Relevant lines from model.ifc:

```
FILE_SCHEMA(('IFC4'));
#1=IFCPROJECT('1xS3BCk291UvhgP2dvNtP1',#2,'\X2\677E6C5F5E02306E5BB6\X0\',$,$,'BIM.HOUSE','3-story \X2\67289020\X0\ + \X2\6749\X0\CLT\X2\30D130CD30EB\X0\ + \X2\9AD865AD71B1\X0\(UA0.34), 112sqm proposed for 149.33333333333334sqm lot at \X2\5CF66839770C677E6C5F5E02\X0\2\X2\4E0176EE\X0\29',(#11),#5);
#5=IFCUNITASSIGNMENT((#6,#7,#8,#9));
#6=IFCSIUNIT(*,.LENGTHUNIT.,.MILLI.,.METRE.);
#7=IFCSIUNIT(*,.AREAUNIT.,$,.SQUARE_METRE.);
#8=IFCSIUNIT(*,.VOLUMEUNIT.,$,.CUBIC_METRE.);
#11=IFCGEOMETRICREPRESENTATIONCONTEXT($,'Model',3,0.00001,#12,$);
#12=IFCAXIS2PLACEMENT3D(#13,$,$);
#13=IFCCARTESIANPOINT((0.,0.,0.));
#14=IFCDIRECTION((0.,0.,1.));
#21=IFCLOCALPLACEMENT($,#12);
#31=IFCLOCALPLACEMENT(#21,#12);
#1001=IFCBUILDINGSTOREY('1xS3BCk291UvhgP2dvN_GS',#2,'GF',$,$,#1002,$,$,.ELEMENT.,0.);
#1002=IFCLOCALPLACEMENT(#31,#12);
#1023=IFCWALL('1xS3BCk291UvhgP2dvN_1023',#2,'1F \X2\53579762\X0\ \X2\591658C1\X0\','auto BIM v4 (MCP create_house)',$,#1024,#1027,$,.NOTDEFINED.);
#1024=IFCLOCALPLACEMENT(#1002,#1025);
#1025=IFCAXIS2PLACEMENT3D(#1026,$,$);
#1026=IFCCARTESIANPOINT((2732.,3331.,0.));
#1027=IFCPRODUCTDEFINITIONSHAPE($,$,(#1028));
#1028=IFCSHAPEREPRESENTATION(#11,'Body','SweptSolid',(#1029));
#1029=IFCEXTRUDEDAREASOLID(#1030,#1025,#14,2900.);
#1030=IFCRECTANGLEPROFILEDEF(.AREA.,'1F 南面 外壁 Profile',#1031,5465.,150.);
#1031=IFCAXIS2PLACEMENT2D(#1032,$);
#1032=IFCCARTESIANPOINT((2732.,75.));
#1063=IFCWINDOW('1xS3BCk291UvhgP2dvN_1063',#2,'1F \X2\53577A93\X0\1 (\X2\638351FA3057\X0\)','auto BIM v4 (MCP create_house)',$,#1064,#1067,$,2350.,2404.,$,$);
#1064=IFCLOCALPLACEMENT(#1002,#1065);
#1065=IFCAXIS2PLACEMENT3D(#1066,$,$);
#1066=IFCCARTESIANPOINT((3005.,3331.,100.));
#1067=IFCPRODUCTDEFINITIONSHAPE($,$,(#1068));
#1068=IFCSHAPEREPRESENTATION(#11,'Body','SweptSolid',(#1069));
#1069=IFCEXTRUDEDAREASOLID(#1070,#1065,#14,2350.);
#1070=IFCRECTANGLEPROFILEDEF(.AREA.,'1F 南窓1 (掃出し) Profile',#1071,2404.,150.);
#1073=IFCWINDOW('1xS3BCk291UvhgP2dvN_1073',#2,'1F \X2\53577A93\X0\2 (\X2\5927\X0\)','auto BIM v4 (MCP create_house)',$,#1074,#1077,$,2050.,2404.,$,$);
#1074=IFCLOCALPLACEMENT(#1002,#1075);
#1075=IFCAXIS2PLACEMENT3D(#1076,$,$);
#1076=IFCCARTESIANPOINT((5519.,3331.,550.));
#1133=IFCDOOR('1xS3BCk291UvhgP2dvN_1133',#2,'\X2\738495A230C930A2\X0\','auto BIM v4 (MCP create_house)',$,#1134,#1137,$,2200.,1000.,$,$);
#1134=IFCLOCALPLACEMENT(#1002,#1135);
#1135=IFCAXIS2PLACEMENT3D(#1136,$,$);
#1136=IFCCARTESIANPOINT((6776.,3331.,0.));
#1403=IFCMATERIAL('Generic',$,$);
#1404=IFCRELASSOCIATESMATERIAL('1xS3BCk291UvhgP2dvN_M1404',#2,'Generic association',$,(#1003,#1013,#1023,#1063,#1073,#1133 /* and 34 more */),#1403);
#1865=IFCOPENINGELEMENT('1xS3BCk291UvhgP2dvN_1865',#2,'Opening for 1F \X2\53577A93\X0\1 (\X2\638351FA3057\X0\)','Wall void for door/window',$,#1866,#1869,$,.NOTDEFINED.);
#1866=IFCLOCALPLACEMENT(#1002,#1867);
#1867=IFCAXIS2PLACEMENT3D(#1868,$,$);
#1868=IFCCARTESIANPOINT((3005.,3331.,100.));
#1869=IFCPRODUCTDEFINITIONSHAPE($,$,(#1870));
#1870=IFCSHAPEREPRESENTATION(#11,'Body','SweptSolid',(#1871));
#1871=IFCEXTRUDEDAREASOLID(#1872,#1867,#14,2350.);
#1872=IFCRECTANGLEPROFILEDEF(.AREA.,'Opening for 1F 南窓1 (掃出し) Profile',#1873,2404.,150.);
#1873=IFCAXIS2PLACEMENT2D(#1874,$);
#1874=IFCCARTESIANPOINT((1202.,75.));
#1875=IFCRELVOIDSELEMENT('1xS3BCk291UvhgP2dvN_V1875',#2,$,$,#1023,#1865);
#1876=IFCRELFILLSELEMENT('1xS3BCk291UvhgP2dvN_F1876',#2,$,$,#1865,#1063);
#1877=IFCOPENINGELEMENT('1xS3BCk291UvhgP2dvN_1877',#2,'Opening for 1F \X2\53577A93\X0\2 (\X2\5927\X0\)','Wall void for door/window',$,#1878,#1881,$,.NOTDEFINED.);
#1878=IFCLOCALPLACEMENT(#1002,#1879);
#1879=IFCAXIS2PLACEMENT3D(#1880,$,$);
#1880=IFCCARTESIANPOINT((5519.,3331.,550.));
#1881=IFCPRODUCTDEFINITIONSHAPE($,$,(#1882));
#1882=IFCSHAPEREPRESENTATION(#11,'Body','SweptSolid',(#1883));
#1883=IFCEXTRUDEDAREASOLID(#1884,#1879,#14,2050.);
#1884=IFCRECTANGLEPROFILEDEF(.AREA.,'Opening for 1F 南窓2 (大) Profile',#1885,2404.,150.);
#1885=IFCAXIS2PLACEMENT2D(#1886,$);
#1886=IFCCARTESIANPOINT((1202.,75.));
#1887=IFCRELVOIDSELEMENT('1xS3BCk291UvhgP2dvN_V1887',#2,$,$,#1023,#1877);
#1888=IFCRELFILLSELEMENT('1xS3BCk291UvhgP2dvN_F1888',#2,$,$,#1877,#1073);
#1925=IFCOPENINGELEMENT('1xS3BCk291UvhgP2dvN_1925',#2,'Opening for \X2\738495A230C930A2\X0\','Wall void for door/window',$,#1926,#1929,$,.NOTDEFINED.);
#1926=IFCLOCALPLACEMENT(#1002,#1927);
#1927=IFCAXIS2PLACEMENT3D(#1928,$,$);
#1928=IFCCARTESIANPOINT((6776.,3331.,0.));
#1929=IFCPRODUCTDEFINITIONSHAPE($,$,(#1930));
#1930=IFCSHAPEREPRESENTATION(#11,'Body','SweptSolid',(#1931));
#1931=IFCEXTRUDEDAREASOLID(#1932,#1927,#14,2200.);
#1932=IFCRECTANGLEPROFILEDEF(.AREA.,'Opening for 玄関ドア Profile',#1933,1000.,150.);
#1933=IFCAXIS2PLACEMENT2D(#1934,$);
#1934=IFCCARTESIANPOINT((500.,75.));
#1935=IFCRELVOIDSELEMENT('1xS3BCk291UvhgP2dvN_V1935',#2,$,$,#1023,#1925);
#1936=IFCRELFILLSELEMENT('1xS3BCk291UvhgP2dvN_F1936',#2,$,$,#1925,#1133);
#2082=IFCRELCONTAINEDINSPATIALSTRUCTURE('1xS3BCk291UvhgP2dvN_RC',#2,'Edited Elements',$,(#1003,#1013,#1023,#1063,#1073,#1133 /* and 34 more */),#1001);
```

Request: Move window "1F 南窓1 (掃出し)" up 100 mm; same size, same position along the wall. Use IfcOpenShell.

```python
import numpy as np
import ifcopenshell
import ifcopenshell.api.geometry
import ifcopenshell.util.placement
import ifcopenshell.util.unit

model = ifcopenshell.open("model.ifc")
unit_scale = ifcopenshell.util.unit.calculate_unit_scale(model)

window = model.by_guid("1xS3BCk291UvhgP2dvN_1063")
opening = window.FillsVoids[0].RelatingOpeningElement
dz = 0.1 / unit_scale

shift = np.array([0.0, 0.0, dz])
# The window is not placed relative to its opening, so move both.
for product in (opening, window):
    matrix = ifcopenshell.util.placement.get_local_placement(product.ObjectPlacement)
    matrix[:3, 3] += shift
    ifcopenshell.api.geometry.edit_object_placement(model, product=product, matrix=matrix, is_si=False)

print(f"moved by {dz * unit_scale:+.3f} m")

model.write("model_edited.ifc")
```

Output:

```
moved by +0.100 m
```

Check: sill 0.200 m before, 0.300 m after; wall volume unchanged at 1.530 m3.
